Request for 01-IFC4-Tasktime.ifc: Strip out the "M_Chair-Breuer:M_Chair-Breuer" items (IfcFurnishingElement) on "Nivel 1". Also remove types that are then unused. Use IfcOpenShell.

First a look at what the model holds.

```python
import ifcopenshell
import ifcopenshell.util.element

model = ifcopenshell.open("01-IFC4-Tasktime.ifc")
print(model.schema)
storey = next(s for s in model.by_type("IfcBuildingStorey") if s.Name == "Nivel 1")
furniture = [e for e in ifcopenshell.util.element.get_decomposition(storey) if e.is_a("IfcFurnishingElement")]
seen = {}
for e in furniture:
    element_type = ifcopenshell.util.element.get_type(e)
    name = element_type.Name if element_type not in (None, e) else None
    seen[name] = seen.get(name, 0) + 1
for name, count in sorted(seen.items(), key=str):
    print(count, "x", name)
```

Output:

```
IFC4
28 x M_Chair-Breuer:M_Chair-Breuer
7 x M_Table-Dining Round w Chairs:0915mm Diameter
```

```python
import ifcopenshell
import ifcopenshell.api.root
import ifcopenshell.util.element

model = ifcopenshell.open("01-IFC4-Tasktime.ifc")

storey = next(s for s in model.by_type("IfcBuildingStorey") if s.Name == "Nivel 1")
furniture = [e for e in ifcopenshell.util.element.get_decomposition(storey) if e.is_a("IfcFurnishingElement")]
targets = [e for e in furniture if (t := ifcopenshell.util.element.get_type(e)) not in (None, e) and t.Name == "M_Chair-Breuer:M_Chair-Breuer"]
types = {ifcopenshell.util.element.get_type(e) for e in targets} - {None, *targets}

for e in targets:
    ifcopenshell.api.root.remove_product(model, product=e)
print(len(targets), "removed")

unused = [t for t in types if not ifcopenshell.util.element.get_types(t)]
for t in unused:
    ifcopenshell.api.root.remove_product(model, product=t)
print(len(unused), "unused types removed")

model.write("01-IFC4-Tasktime-out.ifc")
```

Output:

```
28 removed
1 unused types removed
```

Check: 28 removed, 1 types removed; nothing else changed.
